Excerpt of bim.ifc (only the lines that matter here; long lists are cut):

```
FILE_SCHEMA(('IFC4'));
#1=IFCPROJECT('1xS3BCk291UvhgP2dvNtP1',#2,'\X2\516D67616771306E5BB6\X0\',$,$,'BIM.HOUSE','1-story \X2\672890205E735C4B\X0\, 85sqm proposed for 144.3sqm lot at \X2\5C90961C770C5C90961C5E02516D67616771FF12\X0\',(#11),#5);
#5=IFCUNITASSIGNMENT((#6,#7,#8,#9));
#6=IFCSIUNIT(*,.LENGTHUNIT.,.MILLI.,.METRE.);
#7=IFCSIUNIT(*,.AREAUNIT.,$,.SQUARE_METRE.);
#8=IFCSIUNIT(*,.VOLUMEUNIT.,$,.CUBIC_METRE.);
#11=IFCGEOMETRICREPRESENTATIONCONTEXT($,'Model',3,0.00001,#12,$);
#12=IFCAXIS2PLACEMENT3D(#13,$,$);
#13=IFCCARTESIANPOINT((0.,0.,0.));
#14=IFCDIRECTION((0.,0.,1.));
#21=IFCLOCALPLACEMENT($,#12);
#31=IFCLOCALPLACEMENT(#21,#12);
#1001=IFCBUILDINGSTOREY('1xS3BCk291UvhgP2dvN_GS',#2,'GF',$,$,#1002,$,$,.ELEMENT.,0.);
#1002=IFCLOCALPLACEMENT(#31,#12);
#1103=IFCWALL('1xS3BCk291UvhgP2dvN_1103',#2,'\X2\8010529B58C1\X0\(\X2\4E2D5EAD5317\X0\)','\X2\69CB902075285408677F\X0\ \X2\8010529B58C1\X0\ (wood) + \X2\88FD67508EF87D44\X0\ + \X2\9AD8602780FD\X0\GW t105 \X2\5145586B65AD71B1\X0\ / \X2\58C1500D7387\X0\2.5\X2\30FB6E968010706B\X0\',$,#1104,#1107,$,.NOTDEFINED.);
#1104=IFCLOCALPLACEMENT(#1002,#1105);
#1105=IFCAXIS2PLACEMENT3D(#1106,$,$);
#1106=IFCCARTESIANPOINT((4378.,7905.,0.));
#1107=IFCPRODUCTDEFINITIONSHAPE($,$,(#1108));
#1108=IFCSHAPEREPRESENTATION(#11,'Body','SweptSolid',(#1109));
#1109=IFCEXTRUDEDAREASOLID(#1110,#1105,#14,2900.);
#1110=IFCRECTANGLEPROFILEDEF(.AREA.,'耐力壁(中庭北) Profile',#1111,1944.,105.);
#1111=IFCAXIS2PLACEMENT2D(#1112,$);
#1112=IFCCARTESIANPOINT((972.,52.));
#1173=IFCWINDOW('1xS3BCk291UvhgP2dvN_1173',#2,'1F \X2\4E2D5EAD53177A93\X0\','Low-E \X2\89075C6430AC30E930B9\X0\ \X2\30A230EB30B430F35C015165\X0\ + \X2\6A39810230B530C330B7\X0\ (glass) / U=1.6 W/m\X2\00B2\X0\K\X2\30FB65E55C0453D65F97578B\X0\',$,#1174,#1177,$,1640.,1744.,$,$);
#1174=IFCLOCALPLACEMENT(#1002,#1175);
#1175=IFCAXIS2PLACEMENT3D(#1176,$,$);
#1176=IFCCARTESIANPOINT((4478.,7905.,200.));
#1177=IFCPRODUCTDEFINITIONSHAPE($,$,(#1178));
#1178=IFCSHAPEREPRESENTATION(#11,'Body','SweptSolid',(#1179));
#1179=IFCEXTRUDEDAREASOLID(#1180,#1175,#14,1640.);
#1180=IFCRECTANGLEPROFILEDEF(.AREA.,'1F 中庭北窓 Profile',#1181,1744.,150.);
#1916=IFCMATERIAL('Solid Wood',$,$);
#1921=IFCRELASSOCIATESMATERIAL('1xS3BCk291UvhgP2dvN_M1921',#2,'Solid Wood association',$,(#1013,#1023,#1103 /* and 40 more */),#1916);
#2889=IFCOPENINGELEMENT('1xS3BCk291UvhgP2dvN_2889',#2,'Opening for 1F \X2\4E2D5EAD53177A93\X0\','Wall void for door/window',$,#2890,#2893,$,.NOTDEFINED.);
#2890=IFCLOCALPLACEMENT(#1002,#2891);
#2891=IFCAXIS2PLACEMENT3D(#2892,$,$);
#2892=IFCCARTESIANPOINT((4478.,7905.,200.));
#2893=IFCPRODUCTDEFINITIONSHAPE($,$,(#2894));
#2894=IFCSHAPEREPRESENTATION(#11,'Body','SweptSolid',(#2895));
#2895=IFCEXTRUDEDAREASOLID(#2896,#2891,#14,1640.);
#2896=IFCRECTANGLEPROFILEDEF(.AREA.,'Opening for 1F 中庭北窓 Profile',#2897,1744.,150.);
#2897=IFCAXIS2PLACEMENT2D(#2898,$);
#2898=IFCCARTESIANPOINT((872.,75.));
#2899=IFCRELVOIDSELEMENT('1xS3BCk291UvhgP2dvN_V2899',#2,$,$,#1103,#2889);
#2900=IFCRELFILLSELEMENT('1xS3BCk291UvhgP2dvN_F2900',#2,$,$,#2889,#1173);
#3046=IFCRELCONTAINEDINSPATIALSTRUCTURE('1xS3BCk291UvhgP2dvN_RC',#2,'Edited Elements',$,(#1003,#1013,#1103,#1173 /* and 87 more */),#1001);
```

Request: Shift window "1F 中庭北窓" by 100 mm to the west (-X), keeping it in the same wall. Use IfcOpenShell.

```python
import ifcopenshell
import ifcopenshell.api.geometry
import ifcopenshell.util.placement

model = ifcopenshell.open("bim.ifc")

window = model.by_guid("1xS3BCk291UvhgP2dvN_1173")
opening = window.FillsVoids[0].RelatingOpeningElement
wall = opening.VoidsElements[0].RelatingBuildingElement

wall_matrix = ifcopenshell.util.placement.get_local_placement(wall.ObjectPlacement)
shift = wall_matrix[:3, 0] * -100.0
before = ifcopenshell.util.placement.get_local_placement(window.ObjectPlacement)[:3, 3].copy()

# The window is not placed relative to its opening, so move both.
for product in (opening, window):
    matrix = ifcopenshell.util.placement.get_local_placement(product.ObjectPlacement)
    matrix[:3, 3] += shift
    ifcopenshell.api.geometry.edit_object_placement(model, product=product, matrix=matrix, is_si=False)

after = ifcopenshell.util.placement.get_local_placement(window.ObjectPlacement)[:3, 3]
print("window moved by", (after - before).round(3) + 0.0)

model.write("bim_rev.ifc")
```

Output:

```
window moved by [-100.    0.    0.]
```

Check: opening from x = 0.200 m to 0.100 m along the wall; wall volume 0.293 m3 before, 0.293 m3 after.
